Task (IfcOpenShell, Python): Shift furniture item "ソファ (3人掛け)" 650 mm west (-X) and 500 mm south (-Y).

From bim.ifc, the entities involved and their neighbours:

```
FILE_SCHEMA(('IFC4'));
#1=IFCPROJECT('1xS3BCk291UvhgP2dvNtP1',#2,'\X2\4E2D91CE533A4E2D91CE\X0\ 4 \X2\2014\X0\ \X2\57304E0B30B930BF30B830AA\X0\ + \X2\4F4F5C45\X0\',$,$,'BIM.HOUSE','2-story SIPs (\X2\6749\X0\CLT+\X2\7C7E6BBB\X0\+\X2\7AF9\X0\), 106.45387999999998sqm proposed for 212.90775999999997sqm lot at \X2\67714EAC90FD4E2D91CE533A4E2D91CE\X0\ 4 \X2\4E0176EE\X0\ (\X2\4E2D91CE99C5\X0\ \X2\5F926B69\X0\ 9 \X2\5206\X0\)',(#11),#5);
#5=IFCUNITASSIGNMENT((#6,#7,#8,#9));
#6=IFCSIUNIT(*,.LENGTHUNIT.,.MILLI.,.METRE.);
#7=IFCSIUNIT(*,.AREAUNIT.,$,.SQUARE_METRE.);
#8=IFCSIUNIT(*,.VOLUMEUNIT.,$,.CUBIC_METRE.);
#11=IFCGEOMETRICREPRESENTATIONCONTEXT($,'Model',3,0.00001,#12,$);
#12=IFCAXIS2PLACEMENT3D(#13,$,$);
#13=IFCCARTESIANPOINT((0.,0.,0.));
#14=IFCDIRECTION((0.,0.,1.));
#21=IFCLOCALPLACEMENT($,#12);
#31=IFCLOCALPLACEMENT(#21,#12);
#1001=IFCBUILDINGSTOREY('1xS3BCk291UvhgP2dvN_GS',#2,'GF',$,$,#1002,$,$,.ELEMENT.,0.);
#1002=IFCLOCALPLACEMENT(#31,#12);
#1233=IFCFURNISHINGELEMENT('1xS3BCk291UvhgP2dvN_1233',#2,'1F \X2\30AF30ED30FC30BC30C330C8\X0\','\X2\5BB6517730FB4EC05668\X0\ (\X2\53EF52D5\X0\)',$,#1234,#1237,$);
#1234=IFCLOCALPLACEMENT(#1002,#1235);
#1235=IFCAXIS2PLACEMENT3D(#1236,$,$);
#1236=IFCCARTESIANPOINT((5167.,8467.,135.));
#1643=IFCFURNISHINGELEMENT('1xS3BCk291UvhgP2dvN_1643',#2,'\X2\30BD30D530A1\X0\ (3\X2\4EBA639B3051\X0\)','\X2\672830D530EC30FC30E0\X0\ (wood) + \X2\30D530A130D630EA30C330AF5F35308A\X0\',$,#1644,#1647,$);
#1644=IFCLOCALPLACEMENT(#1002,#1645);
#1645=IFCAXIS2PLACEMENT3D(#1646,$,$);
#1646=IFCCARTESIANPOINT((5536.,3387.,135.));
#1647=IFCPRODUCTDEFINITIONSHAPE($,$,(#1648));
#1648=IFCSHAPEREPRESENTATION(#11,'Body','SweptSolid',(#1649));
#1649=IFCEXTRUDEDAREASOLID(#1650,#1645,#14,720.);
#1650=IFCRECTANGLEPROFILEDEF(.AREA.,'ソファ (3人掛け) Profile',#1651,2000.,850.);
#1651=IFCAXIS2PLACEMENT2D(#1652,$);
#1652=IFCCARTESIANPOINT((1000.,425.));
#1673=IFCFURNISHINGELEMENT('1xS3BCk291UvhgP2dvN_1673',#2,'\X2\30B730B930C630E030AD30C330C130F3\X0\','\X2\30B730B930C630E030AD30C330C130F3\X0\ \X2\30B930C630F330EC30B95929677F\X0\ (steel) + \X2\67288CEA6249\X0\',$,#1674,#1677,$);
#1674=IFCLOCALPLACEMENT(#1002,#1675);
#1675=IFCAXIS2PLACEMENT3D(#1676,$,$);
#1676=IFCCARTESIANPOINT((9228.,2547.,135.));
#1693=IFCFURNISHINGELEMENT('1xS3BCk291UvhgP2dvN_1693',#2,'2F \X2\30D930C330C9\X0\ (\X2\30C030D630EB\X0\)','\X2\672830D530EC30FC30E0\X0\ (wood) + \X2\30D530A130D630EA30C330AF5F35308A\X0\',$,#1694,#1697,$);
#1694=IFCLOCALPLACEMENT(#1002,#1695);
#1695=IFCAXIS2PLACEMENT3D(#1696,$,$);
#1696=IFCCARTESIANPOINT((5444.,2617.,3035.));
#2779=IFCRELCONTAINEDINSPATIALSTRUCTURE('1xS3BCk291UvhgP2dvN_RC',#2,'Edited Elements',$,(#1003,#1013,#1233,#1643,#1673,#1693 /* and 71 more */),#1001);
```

```python
import ifcopenshell
import ifcopenshell.api.geometry
import ifcopenshell.util.placement

model = ifcopenshell.open("bim.ifc")

item = model.by_guid("1xS3BCk291UvhgP2dvN_1643")
matrix = ifcopenshell.util.placement.get_local_placement(item.ObjectPlacement)
matrix[0, 3] -= 650.0
matrix[1, 3] -= 500.0
ifcopenshell.api.geometry.edit_object_placement(model, product=item, matrix=matrix, is_si=False)

print(ifcopenshell.util.placement.get_local_placement(item.ObjectPlacement).round(3) + 0.0)

model.write("bim_rev.ifc")
```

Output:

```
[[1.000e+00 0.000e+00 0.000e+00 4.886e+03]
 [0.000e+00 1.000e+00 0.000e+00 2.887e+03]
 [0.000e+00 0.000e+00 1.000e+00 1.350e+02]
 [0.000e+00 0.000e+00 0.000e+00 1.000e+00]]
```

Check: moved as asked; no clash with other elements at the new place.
